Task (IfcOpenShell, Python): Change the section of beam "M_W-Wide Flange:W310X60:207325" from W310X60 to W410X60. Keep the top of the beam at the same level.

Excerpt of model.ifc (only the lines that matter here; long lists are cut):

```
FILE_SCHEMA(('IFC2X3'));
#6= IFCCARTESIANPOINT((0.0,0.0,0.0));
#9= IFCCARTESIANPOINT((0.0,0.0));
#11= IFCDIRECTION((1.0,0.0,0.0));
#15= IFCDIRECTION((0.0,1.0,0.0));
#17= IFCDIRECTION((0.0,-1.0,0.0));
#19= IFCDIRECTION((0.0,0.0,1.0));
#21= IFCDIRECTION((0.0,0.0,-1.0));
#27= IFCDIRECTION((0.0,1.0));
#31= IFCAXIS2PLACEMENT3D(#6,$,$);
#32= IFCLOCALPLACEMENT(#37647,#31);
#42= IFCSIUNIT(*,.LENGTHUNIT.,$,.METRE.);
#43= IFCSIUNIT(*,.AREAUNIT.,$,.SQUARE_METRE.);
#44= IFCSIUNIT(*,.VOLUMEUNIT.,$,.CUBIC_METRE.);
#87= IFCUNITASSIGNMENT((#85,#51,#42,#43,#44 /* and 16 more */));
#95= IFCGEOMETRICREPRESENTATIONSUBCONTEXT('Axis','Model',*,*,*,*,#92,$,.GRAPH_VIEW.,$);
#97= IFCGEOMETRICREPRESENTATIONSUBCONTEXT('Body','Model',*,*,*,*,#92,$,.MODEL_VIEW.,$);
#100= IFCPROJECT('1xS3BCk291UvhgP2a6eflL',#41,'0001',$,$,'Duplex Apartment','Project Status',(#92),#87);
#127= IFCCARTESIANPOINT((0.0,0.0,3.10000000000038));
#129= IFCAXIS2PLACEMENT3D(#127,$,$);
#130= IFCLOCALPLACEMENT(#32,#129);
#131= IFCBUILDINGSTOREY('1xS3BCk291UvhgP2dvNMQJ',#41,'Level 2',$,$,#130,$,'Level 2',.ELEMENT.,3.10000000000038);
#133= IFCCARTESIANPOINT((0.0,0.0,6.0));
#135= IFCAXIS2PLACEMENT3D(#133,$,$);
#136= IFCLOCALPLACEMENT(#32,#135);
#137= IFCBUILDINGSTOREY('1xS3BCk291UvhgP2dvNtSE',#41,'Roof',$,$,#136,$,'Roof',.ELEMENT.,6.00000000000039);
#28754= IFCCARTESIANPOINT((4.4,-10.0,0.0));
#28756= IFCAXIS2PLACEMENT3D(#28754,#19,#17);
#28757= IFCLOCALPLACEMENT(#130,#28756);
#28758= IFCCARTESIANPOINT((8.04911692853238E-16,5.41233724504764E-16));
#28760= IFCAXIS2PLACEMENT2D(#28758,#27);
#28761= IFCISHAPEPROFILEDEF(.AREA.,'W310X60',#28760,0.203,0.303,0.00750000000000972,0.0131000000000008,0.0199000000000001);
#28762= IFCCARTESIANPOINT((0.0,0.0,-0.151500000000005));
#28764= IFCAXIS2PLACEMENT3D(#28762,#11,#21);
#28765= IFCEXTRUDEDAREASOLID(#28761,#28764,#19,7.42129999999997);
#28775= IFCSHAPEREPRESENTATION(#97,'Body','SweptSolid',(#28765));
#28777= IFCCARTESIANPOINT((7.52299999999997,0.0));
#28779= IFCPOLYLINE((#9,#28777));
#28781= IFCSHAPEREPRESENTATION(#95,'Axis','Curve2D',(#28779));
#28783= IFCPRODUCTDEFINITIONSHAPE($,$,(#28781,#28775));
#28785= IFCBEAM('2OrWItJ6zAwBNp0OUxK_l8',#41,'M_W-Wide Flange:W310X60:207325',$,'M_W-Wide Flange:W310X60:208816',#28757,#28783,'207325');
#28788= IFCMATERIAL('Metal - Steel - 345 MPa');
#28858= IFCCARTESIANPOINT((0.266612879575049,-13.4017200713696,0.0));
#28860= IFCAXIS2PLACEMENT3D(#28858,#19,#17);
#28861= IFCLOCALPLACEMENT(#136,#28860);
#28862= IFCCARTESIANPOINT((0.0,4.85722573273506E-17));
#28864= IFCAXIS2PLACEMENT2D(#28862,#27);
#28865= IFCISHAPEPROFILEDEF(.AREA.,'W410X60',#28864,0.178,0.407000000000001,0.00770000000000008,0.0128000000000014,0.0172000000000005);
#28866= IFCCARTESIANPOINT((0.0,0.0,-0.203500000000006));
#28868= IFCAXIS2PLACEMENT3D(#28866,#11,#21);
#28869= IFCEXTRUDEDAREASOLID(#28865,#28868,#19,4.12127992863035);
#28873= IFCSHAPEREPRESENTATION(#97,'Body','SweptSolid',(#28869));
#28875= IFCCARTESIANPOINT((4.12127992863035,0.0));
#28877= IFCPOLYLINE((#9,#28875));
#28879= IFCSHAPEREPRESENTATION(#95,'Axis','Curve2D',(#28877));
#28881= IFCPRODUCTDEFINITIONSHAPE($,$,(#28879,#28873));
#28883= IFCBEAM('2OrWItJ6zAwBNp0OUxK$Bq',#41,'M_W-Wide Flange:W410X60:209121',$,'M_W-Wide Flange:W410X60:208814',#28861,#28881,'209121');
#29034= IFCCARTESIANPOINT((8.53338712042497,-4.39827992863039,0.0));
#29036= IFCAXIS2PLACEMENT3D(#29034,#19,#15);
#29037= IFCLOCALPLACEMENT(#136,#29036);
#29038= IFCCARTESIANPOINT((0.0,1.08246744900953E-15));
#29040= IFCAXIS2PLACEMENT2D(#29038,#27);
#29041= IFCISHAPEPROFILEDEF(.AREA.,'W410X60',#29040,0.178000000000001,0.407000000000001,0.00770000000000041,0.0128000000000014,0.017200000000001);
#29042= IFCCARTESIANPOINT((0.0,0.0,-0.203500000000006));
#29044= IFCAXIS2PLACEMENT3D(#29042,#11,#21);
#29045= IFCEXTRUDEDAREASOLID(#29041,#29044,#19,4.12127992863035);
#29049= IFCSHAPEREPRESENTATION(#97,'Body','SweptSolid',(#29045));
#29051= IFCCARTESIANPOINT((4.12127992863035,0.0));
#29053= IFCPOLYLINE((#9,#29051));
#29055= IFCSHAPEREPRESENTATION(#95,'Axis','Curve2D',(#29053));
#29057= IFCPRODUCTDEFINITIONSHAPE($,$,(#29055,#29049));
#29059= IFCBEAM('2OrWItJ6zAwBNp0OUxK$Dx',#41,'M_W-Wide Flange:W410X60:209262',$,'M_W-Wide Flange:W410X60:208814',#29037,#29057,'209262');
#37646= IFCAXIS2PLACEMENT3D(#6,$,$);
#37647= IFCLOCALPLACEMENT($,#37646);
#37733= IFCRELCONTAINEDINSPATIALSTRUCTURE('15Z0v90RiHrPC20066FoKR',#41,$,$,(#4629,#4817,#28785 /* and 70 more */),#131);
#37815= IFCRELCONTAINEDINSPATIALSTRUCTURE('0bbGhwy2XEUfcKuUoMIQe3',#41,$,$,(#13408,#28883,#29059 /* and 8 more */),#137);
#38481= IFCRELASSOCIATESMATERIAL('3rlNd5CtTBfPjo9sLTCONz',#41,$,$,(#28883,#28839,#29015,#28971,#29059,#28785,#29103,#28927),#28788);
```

```python
import ifcopenshell
import ifcopenshell.util.element
import ifcopenshell.util.representation

model = ifcopenshell.open("model.ifc")

member = model.by_guid("2OrWItJ6zAwBNp0OUxK_l8")
source = next(p for p in model.by_type("IfcIShapeProfileDef") if p.ProfileName == "W410X60")

body = ifcopenshell.util.representation.get_representation(member, "Model", "Body")
solid = body.Items[0]
old_profile = solid.SweptArea

# Copy the section's sizes but keep this member's own profile position.
profile = ifcopenshell.util.element.copy(model, source)
# Profiles are centred, so shift by half the change in depth to hold the top.
shift = (old_profile.OverallDepth - profile.OverallDepth) / 2
x, y = old_profile.Position.Location.Coordinates
up = (-1.0, 0.0)  # upwards, in the solid's own plane
location = model.createIfcCartesianPoint((x + up[0] * shift, y + up[1] * shift))
profile.Position = model.createIfcAxis2Placement2D(location, old_profile.Position.RefDirection)
solid.SweptArea = profile
if not model.get_total_inverses(old_profile):
    ifcopenshell.util.element.remove_deep2(model, old_profile)
member.Name = member.Name.replace("W310X60", "W410X60")
member.ObjectType = member.ObjectType.replace("W310X60", "W410X60")

print(solid.SweptArea)

model.write("model_v2.ifc")
```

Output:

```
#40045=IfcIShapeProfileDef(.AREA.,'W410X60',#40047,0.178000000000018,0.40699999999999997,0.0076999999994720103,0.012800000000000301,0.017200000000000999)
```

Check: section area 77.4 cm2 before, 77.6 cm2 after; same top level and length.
